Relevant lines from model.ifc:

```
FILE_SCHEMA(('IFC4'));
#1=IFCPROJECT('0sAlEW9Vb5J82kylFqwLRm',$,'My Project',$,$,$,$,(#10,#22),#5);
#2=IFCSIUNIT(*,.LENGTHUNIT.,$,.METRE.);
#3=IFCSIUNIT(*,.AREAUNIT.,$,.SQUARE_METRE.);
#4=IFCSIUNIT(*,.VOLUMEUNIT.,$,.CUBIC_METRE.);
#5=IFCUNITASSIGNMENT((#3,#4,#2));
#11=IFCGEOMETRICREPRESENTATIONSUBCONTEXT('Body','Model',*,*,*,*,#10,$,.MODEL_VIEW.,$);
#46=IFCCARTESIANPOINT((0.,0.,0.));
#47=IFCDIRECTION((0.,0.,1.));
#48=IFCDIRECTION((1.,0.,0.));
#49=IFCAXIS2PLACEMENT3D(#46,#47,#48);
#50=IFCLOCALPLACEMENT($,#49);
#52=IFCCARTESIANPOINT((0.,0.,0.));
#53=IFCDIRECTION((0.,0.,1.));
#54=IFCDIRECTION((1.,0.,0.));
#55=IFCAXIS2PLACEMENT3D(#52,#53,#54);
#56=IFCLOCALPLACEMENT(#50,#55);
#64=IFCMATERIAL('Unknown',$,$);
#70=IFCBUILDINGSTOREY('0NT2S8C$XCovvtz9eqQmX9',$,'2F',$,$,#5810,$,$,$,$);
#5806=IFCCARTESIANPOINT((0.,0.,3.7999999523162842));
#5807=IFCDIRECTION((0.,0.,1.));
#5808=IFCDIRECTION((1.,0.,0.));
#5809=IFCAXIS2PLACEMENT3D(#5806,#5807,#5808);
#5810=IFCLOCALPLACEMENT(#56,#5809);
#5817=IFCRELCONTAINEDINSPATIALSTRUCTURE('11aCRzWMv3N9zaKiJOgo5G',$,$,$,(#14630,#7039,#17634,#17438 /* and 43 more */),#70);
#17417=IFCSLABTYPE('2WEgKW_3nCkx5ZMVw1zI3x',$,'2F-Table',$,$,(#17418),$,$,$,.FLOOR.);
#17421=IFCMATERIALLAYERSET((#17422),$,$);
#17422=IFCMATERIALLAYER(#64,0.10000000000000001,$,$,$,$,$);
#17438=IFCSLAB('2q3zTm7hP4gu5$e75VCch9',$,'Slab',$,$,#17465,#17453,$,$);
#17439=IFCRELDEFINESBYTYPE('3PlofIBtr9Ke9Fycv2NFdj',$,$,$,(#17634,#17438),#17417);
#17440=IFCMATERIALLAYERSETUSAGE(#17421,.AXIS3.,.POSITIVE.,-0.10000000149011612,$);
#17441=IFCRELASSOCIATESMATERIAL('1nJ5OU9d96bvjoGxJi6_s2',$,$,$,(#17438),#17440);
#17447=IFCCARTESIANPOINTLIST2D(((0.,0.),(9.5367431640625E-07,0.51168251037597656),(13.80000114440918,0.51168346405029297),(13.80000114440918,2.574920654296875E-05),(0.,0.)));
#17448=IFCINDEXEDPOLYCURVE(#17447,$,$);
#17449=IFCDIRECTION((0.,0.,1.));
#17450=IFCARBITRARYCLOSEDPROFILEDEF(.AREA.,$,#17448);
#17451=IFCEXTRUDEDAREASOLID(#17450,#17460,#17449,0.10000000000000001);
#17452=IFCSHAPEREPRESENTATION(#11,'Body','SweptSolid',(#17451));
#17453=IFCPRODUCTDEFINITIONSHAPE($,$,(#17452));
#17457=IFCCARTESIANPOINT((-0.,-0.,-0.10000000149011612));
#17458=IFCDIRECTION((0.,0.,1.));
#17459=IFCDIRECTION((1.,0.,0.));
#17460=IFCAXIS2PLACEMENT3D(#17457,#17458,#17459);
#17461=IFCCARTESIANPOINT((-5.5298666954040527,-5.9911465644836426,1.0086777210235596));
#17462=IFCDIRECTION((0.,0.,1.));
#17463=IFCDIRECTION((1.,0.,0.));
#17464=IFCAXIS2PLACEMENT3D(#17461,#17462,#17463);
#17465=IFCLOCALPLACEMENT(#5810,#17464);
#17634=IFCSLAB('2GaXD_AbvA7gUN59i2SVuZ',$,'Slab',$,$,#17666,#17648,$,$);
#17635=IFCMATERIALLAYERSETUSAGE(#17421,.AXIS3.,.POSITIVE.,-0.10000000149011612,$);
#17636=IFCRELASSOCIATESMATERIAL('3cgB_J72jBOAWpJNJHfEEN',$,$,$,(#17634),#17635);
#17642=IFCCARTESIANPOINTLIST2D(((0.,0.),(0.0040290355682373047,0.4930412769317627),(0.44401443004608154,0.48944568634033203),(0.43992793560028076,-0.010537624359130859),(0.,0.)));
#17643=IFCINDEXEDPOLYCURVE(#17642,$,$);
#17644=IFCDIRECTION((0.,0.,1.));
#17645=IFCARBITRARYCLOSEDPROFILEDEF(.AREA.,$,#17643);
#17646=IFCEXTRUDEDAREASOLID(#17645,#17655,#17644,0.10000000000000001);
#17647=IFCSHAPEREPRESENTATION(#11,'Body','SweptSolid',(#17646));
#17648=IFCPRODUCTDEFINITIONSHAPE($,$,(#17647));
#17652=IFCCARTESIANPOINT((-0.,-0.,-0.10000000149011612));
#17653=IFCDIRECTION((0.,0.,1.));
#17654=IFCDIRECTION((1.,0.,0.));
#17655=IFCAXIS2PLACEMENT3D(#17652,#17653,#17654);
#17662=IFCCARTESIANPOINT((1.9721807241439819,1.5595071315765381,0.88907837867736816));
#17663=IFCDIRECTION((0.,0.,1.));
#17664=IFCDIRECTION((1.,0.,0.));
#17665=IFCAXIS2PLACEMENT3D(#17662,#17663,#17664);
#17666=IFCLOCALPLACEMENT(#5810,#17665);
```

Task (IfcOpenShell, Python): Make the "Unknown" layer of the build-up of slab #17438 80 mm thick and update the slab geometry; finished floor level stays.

```python
import ifcopenshell
import ifcopenshell.util.element
import ifcopenshell.util.representation

model = ifcopenshell.open("model.ifc")

layer_set = model.by_id(17421)
layer = next(l for l in layer_set.MaterialLayers if l.Material and l.Material.Name == "Unknown")
change = 0.08 - layer.LayerThickness
layer.LayerThickness += change

# The layer set is shared, so every slab that uses it gets the new thickness.
slabs = [e for e in ifcopenshell.util.element.get_elements_by_material(model, layer_set) if e.is_a("IfcSlab")]
for slab in sorted(slabs, key=lambda e: e.id()):
    body = ifcopenshell.util.representation.get_representation(slab, "Model", "Body")
    solid = body.Items[0]
    old_depth = solid.Depth
    solid.Depth += change
    # Extruded upwards: lower the start of the extrusion so the top stays.
    x, y, z = solid.Position.Location.Coordinates
    solid.Position.Location = model.createIfcCartesianPoint((x, y, z - change))
    print(slab.id(), f"{old_depth:g} -> {solid.Depth:g}")

# The layers are counted up from the underside, which has moved.
for usage in {ifcopenshell.util.element.get_material(slab) for slab in slabs}:
    usage.OffsetFromReferenceLine -= change

model.write("model_rev.ifc")
```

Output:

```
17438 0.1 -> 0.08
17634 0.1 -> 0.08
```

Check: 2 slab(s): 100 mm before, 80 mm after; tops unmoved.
